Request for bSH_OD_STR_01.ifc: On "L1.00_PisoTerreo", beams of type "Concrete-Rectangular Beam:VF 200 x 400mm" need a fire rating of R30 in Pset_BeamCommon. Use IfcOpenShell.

First a look at what the model holds.

```python
import ifcopenshell
import ifcopenshell.util.element

model = ifcopenshell.open("bSH_OD_STR_01.ifc")
print(model.schema)
storey = next(s for s in model.by_type("IfcBuildingStorey") if s.Name == "L1.00_PisoTerreo")
beams = [e for e in ifcopenshell.util.element.get_decomposition(storey) if e.is_a("IfcBeam")]
seen = {}
for e in beams:
    element_type = ifcopenshell.util.element.get_type(e)
    key = (element_type.Name if element_type != e and element_type else None, ifcopenshell.util.element.get_pset(e, "Pset_BeamCommon", "FireRating"))
    seen[key] = seen.get(key, 0) + 1
for (name, value), count in sorted(seen.items(), key=str):
    print(count, "x", name, "|", value)
```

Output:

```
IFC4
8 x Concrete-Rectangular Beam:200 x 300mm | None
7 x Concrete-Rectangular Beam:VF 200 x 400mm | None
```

```python
import ifcopenshell
import ifcopenshell.api.pset
import ifcopenshell.util.element

model = ifcopenshell.open("bSH_OD_STR_01.ifc")

storey = next(s for s in model.by_type("IfcBuildingStorey") if s.Name == "L1.00_PisoTerreo")
beams = [e for e in ifcopenshell.util.element.get_decomposition(storey) if e.is_a("IfcBeam")]

count = 0
for e in beams:
    element_type = ifcopenshell.util.element.get_type(e)
    if element_type in (None, e) or element_type.Name != "Concrete-Rectangular Beam:VF 200 x 400mm":
        continue
    # add_pset returns the element's existing set when there is one.
    pset = ifcopenshell.api.pset.add_pset(model, product=e, name="Pset_BeamCommon")
    ifcopenshell.api.pset.edit_pset(model, pset=pset, properties={"FireRating": "R30"})
    count += 1

print(count, "beams updated")

model.write("bSH_OD_STR_01_rev.ifc")
```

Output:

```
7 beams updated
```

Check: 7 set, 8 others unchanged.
